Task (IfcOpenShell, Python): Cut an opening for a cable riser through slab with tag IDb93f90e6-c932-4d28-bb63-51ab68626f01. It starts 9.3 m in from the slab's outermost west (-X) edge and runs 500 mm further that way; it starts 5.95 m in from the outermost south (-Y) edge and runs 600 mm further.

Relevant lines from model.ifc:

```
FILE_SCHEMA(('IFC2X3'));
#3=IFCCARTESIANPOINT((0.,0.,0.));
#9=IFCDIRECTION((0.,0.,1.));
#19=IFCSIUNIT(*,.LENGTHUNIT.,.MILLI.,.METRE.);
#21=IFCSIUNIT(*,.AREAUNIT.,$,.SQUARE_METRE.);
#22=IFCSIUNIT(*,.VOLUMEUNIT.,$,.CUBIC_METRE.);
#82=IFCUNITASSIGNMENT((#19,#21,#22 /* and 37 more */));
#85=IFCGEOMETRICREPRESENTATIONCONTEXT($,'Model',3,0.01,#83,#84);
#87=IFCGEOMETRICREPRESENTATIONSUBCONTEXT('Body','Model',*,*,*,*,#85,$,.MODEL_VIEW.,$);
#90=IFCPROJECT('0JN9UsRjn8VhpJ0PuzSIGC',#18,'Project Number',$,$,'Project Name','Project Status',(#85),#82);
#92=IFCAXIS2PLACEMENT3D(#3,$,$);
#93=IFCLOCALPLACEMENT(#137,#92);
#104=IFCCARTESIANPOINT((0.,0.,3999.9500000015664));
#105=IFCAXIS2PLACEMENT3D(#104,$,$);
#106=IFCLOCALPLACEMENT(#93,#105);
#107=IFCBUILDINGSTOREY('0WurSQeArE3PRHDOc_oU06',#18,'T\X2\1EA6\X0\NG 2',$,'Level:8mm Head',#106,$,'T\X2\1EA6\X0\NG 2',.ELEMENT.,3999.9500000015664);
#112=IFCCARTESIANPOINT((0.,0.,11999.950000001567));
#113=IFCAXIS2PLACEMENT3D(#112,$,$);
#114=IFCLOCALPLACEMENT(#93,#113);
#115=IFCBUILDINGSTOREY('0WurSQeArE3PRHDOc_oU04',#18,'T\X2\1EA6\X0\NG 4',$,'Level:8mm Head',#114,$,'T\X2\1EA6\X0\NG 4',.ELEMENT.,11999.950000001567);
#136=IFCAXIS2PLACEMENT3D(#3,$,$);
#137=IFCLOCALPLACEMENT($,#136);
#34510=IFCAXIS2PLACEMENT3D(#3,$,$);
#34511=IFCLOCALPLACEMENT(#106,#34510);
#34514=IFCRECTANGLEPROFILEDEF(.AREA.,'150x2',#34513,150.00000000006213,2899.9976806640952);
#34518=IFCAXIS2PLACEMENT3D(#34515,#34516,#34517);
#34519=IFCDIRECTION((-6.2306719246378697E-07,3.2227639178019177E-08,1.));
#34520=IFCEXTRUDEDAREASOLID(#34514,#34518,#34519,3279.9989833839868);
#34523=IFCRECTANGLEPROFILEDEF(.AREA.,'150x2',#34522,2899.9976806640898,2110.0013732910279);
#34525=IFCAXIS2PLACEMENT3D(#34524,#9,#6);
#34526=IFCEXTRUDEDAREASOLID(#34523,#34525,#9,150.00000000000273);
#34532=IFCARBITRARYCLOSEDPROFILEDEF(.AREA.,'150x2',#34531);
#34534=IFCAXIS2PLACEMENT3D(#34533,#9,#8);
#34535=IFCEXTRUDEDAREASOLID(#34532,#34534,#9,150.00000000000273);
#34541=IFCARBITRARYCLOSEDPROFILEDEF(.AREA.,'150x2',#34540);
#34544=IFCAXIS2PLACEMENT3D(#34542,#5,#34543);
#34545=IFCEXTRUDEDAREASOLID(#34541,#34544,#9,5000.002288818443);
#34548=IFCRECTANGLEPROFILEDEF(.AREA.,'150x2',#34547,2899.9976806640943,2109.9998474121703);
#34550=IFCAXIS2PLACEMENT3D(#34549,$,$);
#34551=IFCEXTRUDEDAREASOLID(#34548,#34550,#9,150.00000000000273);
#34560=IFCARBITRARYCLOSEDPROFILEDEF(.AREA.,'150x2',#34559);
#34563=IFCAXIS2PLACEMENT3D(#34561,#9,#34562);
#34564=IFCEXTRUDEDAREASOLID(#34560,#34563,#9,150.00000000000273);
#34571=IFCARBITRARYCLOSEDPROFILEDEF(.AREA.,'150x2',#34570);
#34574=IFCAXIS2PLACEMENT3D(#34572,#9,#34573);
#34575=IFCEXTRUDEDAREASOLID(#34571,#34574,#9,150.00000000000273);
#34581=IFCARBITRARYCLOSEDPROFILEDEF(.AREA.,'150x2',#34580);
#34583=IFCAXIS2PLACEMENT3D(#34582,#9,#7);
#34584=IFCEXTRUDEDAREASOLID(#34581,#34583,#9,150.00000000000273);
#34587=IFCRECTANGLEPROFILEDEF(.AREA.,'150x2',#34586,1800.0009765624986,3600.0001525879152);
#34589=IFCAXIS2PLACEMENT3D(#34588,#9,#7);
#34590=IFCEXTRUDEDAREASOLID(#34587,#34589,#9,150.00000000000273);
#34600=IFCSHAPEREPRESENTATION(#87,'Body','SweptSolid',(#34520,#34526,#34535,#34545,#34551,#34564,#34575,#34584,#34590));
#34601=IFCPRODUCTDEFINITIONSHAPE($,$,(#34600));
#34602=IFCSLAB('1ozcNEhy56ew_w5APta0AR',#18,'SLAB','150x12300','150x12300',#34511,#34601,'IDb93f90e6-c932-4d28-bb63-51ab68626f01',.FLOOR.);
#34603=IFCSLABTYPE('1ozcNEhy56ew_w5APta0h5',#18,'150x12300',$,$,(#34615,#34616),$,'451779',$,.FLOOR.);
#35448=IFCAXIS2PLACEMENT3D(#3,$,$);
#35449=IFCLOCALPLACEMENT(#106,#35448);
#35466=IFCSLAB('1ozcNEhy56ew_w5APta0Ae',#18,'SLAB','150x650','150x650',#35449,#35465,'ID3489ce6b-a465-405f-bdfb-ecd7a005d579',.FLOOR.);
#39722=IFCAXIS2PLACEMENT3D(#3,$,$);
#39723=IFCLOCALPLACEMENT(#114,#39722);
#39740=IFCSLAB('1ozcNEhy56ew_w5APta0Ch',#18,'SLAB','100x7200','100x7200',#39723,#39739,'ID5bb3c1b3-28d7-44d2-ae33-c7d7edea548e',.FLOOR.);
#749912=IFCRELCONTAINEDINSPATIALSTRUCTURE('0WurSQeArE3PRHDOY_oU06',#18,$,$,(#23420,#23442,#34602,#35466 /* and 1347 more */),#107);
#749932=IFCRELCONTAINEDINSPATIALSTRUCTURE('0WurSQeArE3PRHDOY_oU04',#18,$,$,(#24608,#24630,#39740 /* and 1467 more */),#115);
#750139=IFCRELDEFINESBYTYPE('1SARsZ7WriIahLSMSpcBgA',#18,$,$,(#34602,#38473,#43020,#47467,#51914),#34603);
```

```python
import numpy as np
import ifcopenshell
import ifcopenshell.api.feature
import ifcopenshell.api.geometry
import ifcopenshell.api.root
import ifcopenshell.geom
import ifcopenshell.util.placement
import ifcopenshell.util.representation
import ifcopenshell.util.shape
import ifcopenshell.util.unit

model = ifcopenshell.open("model.ifc")
unit_scale = ifcopenshell.util.unit.calculate_unit_scale(model)
settings = ifcopenshell.geom.settings()


def volume(element):
    """Net volume in cubic metres, openings subtracted."""
    shape = ifcopenshell.geom.create_shape(settings, element)
    return ifcopenshell.util.shape.get_volume(shape.geometry)


slab = model.by_guid("1ozcNEhy56ew_w5APta0AR")
before = volume(slab)

# Extent in the slab's own axes, in metres. The edges named are its -X and -Y sides.
slab_shape = ifcopenshell.geom.create_shape(settings, slab)
vertices = ifcopenshell.util.shape.get_vertices(slab_shape.geometry)
x_min, y_min, bottom = vertices.min(axis=0)
top = vertices[:, 2].max()

opening = ifcopenshell.api.root.create_entity(model, ifc_class="IfcOpeningElement", name="Cable riser opening")
context = ifcopenshell.util.representation.get_context(model, "Model", "Body", "MODEL_VIEW")
width, depth = 0.5, 0.6
outline = [(0.0, 0.0), (width, 0.0), (width, depth), (0.0, depth), (0.0, 0.0)]
# Overshoot both faces by 50 mm so the cut is clean.
shape = ifcopenshell.api.geometry.add_slab_representation(
    model, context=context, depth=top - bottom + 0.1, polyline=outline
)
ifcopenshell.api.geometry.assign_representation(model, product=opening, representation=shape)

matrix = ifcopenshell.util.placement.get_local_placement(slab.ObjectPlacement)
matrix[:, 3] = matrix @ np.append(np.array([x_min + 9.3, y_min + 5.95, bottom - 0.05]) / unit_scale, 1.0)
ifcopenshell.api.geometry.edit_object_placement(model, product=opening, matrix=matrix, is_si=False)
ifcopenshell.api.feature.add_feature(model, feature=opening, element=slab)

after = volume(slab)

print(f"slab volume {before:.3f} -> {after:.3f} m3")

model.write("model_rev.ifc")
```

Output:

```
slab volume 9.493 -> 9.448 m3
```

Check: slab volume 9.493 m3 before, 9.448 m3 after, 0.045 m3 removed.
